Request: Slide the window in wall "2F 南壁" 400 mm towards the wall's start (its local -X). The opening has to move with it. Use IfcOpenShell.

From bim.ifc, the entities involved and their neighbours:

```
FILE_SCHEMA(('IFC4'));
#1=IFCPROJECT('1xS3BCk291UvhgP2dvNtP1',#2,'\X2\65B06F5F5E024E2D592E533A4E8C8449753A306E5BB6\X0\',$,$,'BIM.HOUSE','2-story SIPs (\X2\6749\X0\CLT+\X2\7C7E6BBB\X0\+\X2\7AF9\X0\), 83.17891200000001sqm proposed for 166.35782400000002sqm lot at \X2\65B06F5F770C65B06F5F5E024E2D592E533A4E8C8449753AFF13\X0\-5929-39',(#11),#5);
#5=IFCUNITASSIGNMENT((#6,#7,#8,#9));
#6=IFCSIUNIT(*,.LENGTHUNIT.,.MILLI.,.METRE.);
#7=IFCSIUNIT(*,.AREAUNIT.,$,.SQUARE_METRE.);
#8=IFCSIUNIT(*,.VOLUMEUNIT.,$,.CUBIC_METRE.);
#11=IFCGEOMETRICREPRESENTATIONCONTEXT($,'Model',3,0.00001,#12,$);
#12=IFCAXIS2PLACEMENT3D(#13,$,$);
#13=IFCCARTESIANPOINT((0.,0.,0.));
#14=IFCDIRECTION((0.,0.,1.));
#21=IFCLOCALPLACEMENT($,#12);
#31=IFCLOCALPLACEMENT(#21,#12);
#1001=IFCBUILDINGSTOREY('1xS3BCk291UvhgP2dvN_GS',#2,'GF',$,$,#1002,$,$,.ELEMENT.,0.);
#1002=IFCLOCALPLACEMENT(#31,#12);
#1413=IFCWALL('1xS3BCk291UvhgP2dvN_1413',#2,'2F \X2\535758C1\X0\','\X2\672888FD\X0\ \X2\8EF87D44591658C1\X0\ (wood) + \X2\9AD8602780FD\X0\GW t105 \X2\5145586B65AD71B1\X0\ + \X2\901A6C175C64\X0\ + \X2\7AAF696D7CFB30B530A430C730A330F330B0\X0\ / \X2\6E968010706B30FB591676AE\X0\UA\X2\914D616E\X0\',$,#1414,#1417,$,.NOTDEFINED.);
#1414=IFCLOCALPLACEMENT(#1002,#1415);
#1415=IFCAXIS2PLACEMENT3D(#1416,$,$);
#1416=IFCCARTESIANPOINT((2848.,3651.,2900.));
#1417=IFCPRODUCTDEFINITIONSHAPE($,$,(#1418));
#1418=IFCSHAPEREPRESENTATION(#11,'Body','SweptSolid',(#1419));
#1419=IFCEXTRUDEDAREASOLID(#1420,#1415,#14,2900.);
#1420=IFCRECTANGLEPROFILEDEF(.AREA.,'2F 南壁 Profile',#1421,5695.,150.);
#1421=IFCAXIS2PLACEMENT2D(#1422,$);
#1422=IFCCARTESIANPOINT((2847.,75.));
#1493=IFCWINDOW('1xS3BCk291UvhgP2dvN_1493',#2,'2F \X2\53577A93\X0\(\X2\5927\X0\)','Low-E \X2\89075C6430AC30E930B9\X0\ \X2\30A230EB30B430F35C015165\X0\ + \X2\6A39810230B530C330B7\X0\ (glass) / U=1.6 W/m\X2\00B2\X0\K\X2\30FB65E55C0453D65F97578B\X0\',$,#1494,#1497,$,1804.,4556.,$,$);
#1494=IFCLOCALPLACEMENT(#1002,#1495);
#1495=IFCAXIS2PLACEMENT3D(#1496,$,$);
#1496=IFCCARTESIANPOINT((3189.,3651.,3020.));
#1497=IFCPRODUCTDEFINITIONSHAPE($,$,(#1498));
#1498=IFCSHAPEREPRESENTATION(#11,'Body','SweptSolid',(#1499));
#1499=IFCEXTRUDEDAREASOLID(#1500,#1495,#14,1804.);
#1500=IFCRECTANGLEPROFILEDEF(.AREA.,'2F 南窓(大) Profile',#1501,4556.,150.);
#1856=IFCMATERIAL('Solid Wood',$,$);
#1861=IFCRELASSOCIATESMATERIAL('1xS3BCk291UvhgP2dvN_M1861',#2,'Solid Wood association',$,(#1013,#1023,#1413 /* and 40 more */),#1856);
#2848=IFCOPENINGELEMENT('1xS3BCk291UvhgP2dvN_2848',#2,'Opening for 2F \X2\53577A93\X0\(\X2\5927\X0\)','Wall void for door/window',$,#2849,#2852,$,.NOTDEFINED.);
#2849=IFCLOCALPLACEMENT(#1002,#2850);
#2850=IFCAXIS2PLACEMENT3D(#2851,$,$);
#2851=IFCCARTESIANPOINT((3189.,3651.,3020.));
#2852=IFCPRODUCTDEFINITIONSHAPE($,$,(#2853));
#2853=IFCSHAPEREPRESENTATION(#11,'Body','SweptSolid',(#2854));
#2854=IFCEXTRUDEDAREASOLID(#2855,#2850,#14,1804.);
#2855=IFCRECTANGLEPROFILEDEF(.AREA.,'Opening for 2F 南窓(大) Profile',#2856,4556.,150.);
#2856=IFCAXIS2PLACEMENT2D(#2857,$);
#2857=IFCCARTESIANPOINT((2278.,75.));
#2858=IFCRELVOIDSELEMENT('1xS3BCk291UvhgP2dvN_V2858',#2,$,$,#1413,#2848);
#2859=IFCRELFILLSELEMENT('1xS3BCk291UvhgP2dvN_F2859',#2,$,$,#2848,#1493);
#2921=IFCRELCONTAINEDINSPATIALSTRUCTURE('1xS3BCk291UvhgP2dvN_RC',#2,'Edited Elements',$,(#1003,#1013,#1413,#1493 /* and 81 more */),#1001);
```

```python
import ifcopenshell
import ifcopenshell.api.geometry
import ifcopenshell.util.placement

model = ifcopenshell.open("bim.ifc")

window = model.by_guid("1xS3BCk291UvhgP2dvN_1493")
opening = window.FillsVoids[0].RelatingOpeningElement
wall = opening.VoidsElements[0].RelatingBuildingElement

wall_matrix = ifcopenshell.util.placement.get_local_placement(wall.ObjectPlacement)
shift = wall_matrix[:3, 0] * -400.0
before = ifcopenshell.util.placement.get_local_placement(window.ObjectPlacement)[:3, 3].copy()

# The window is not placed relative to its opening, so move both.
for product in (opening, window):
    matrix = ifcopenshell.util.placement.get_local_placement(product.ObjectPlacement)
    matrix[:3, 3] += shift
    ifcopenshell.api.geometry.edit_object_placement(model, product=product, matrix=matrix, is_si=False)

after = ifcopenshell.util.placement.get_local_placement(window.ObjectPlacement)[:3, 3]
print("window moved by", (after - before).round(3) + 0.0)

model.write("bim-out.ifc")
```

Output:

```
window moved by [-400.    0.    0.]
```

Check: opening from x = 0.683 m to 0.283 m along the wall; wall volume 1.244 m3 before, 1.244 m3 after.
